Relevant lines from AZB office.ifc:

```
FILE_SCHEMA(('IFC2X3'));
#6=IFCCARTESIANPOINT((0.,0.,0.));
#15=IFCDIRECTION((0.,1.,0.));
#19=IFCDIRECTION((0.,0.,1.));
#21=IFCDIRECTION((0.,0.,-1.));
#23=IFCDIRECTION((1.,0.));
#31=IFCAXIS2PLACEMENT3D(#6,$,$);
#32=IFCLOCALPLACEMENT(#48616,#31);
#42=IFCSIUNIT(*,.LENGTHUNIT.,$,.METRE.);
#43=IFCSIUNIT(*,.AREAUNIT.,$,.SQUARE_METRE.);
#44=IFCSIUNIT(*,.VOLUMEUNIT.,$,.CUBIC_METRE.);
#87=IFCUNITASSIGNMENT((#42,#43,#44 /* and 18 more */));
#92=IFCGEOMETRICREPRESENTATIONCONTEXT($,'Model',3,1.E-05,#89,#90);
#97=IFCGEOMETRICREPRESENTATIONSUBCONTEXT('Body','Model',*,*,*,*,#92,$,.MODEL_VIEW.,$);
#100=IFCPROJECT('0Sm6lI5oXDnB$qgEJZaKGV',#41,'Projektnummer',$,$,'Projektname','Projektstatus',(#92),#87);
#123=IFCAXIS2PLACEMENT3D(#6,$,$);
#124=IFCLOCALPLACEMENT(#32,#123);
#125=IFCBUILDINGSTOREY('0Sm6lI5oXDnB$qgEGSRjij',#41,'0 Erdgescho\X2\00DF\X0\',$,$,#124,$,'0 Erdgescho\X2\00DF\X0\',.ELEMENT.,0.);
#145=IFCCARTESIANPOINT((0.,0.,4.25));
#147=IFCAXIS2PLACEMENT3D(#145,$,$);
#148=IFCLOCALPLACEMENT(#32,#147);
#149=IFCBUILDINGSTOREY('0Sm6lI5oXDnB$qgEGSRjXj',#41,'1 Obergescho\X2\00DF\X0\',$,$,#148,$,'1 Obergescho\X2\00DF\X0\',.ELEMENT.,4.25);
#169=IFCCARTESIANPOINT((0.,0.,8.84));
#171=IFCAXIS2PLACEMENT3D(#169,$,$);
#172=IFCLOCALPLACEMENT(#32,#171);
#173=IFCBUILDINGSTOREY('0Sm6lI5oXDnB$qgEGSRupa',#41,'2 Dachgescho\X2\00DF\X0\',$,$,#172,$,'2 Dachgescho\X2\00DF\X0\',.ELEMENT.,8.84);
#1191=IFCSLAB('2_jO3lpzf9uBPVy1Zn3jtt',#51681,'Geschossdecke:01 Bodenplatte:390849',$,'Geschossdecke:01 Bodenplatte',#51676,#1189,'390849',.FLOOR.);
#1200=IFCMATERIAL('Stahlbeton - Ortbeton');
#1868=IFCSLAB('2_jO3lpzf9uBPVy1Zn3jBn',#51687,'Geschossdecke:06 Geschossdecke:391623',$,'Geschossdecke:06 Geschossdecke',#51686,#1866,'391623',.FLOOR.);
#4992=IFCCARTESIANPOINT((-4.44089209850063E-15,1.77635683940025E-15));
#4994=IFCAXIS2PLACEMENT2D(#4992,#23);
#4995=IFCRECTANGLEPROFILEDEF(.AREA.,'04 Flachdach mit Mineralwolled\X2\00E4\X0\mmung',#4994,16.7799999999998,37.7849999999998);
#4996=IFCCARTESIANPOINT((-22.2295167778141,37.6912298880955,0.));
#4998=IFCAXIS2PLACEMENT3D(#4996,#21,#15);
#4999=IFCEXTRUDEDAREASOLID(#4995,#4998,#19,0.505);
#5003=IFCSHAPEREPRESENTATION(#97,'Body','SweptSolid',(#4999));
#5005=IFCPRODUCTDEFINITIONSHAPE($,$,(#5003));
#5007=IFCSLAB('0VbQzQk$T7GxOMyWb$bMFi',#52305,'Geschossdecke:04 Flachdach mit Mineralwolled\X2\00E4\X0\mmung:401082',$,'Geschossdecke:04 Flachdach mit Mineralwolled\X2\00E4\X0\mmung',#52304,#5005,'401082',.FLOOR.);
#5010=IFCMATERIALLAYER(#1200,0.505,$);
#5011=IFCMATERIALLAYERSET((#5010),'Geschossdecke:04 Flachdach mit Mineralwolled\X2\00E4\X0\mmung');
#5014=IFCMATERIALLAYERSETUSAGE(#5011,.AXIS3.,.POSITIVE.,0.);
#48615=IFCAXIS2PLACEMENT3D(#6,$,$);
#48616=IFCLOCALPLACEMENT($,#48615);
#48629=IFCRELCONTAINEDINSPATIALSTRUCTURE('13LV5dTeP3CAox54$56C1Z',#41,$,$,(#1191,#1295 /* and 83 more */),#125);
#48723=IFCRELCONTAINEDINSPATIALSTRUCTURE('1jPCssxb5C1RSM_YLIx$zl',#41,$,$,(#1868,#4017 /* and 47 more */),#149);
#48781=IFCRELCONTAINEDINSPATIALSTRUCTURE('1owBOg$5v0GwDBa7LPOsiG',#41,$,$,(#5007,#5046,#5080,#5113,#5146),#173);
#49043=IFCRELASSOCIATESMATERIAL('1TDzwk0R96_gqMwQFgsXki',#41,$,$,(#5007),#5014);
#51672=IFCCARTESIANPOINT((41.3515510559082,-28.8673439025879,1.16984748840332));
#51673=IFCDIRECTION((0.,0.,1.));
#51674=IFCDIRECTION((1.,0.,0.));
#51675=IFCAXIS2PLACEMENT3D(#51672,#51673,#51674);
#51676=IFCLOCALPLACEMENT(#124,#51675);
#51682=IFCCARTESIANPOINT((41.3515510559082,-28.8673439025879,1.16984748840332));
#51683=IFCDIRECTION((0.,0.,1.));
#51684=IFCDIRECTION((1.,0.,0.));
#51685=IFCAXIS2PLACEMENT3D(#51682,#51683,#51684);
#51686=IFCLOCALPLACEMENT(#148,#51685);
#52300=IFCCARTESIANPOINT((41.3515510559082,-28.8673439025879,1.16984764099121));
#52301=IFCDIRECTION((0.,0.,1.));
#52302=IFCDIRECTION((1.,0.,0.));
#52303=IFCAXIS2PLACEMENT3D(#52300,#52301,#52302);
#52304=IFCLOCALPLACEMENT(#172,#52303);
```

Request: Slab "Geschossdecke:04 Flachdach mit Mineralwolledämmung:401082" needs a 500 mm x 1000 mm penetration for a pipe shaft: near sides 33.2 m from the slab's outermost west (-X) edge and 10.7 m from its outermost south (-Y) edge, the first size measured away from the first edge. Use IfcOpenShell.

```python
import numpy as np
import ifcopenshell
import ifcopenshell.api.feature
import ifcopenshell.api.geometry
import ifcopenshell.api.root
import ifcopenshell.geom
import ifcopenshell.util.placement
import ifcopenshell.util.representation
import ifcopenshell.util.shape
import ifcopenshell.util.unit

model = ifcopenshell.open("AZB office.ifc")
unit_scale = ifcopenshell.util.unit.calculate_unit_scale(model)
settings = ifcopenshell.geom.settings()


def volume(element):
    """Net volume in cubic metres, openings subtracted."""
    shape = ifcopenshell.geom.create_shape(settings, element)
    return ifcopenshell.util.shape.get_volume(shape.geometry)


slab = model.by_id(5007)
before = volume(slab)

# Extent in the slab's own axes, in metres. The edges named are its -X and -Y sides.
slab_shape = ifcopenshell.geom.create_shape(settings, slab)
vertices = ifcopenshell.util.shape.get_vertices(slab_shape.geometry)
x_min, y_min, bottom = vertices.min(axis=0)
top = vertices[:, 2].max()

opening = ifcopenshell.api.root.create_entity(model, ifc_class="IfcOpeningElement", name="Pipe shaft opening")
context = ifcopenshell.util.representation.get_context(model, "Model", "Body", "MODEL_VIEW")
width, depth = 0.5, 1
outline = [(0.0, 0.0), (width, 0.0), (width, depth), (0.0, depth), (0.0, 0.0)]
# Overshoot both faces by 50 mm so the cut is clean.
shape = ifcopenshell.api.geometry.add_slab_representation(
    model, context=context, depth=top - bottom + 0.1, polyline=outline
)
ifcopenshell.api.geometry.assign_representation(model, product=opening, representation=shape)

matrix = ifcopenshell.util.placement.get_local_placement(slab.ObjectPlacement)
matrix[:, 3] = matrix @ np.append(np.array([x_min + 33.2, y_min + 10.7, bottom - 0.05]) / unit_scale, 1.0)
ifcopenshell.api.geometry.edit_object_placement(model, product=opening, matrix=matrix, is_si=False)
ifcopenshell.api.feature.add_feature(model, feature=opening, element=slab)

after = volume(slab)

print(f"slab volume {before:.3f} -> {after:.3f} m3")

model.write("AZB office_edited.ifc")
```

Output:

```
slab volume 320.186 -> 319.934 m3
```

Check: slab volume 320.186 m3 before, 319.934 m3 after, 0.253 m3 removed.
